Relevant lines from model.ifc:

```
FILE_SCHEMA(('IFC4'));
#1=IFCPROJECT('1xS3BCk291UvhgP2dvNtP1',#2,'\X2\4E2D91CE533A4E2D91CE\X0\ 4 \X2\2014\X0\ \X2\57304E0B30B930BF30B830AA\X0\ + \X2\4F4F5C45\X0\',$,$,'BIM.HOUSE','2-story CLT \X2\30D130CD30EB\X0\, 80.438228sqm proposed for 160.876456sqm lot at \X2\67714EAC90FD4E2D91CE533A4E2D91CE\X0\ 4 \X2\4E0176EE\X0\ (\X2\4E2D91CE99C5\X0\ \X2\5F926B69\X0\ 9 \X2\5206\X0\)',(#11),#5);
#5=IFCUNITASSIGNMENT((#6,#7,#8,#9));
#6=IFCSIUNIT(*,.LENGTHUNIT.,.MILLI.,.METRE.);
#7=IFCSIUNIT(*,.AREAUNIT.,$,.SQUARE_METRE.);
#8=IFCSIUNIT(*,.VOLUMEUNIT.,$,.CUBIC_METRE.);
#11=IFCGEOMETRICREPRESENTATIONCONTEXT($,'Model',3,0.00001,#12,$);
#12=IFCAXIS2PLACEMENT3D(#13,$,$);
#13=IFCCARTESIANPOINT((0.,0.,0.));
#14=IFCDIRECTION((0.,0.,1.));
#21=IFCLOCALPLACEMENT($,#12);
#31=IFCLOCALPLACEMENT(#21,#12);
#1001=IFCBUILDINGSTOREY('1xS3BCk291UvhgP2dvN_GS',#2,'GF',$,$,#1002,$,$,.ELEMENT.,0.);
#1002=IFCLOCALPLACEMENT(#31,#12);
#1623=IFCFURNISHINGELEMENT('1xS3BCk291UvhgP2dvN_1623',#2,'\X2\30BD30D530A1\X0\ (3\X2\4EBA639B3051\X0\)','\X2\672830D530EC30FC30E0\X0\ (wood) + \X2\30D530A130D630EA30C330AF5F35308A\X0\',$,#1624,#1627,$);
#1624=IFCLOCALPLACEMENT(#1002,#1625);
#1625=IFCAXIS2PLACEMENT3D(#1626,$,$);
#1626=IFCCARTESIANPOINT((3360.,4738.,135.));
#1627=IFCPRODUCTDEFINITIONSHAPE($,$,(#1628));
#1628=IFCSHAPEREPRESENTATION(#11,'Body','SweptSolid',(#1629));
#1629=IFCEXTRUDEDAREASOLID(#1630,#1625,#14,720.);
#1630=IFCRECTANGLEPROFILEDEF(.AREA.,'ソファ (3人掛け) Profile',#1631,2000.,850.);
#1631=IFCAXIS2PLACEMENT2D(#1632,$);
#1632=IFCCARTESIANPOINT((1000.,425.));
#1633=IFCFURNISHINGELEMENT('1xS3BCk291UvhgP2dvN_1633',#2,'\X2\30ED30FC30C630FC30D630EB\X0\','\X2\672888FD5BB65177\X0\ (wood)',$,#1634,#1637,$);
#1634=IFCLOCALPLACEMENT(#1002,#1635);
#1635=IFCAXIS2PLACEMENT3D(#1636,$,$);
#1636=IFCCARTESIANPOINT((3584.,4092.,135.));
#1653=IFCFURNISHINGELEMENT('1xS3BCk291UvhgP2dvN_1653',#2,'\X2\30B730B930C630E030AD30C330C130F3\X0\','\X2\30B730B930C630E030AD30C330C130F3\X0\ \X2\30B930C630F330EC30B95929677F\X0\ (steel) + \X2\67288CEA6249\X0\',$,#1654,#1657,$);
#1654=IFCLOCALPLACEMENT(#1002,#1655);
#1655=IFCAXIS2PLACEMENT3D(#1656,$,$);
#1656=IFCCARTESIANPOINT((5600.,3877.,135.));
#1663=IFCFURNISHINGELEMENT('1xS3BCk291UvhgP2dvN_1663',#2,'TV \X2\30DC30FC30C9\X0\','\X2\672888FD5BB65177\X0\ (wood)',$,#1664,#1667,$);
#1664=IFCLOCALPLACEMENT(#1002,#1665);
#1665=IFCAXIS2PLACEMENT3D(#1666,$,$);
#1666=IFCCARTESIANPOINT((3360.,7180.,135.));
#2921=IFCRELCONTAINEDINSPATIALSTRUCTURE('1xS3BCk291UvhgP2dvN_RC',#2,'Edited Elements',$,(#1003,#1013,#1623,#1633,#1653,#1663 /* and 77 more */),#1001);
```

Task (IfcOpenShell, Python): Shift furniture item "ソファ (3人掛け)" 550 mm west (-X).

```python
import ifcopenshell
import ifcopenshell.api.geometry
import ifcopenshell.util.placement
import ifcopenshell.util.unit

model = ifcopenshell.open("model.ifc")
unit_scale = ifcopenshell.util.unit.calculate_unit_scale(model)

item = model.by_guid("1xS3BCk291UvhgP2dvN_1623")
matrix = ifcopenshell.util.placement.get_local_placement(item.ObjectPlacement)
matrix[0, 3] -= 0.55 / unit_scale
ifcopenshell.api.geometry.edit_object_placement(model, product=item, matrix=matrix, is_si=False)

print(ifcopenshell.util.placement.get_local_placement(item.ObjectPlacement).round(3) + 0.0)

model.write("model-out.ifc")
```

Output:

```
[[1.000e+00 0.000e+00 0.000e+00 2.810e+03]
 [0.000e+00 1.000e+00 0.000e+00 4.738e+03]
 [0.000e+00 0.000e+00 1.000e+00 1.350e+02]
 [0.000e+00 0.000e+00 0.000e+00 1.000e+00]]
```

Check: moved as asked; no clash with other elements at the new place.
